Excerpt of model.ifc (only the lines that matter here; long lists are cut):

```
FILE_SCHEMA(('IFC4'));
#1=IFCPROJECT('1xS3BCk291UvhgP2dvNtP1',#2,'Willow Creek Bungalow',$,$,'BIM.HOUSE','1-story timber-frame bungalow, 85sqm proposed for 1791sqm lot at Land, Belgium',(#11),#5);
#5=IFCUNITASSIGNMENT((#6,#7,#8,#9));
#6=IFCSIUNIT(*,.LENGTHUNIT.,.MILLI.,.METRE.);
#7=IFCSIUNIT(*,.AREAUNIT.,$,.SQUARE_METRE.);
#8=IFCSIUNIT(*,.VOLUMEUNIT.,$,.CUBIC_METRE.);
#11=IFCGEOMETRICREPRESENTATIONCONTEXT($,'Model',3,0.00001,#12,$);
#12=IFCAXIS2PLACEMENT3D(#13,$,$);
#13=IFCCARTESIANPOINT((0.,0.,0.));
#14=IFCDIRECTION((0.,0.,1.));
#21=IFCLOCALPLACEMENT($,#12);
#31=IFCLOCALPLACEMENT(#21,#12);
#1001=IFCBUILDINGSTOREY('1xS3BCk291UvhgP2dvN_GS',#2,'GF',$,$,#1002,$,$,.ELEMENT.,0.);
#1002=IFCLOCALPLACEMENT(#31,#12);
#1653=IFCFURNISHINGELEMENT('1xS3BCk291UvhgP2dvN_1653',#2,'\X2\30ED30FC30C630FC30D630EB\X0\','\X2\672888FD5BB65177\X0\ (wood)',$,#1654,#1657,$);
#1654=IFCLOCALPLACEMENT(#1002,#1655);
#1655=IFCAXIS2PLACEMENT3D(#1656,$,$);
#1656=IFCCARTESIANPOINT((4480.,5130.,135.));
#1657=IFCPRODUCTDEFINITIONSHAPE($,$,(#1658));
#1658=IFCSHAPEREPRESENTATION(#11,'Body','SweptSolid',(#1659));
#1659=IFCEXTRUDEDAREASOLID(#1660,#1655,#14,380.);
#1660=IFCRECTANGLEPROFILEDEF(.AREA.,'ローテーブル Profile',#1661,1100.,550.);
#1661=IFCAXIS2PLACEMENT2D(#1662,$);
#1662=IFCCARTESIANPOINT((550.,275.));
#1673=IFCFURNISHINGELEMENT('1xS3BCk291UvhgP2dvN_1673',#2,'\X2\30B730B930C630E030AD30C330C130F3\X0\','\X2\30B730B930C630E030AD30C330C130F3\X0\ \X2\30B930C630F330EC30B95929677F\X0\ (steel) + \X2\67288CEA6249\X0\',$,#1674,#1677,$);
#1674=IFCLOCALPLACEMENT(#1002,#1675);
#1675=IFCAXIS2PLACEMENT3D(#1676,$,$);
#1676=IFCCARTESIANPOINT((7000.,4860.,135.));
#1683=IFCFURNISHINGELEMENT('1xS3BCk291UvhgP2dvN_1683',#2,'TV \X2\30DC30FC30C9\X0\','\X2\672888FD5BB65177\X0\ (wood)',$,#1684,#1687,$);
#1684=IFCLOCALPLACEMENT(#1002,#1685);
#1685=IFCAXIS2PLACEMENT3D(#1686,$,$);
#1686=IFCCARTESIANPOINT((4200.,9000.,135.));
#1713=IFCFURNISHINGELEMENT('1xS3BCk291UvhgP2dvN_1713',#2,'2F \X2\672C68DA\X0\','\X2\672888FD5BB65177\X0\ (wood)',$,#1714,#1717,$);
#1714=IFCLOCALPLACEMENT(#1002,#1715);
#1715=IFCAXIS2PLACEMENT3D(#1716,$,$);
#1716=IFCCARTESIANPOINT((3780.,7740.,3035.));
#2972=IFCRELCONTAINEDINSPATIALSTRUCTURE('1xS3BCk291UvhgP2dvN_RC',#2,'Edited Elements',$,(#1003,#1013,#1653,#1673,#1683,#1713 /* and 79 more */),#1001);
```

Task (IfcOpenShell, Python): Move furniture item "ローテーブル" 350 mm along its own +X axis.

```python
import ifcopenshell
import ifcopenshell.api.geometry
import ifcopenshell.util.placement
import ifcopenshell.util.unit

model = ifcopenshell.open("model.ifc")
unit_scale = ifcopenshell.util.unit.calculate_unit_scale(model)

item = model.by_guid("1xS3BCk291UvhgP2dvN_1653")
matrix = ifcopenshell.util.placement.get_local_placement(item.ObjectPlacement)
matrix[:3, 3] += matrix[:3, 0] * 0.35 / unit_scale
ifcopenshell.api.geometry.edit_object_placement(model, product=item, matrix=matrix, is_si=False)

print(ifcopenshell.util.placement.get_local_placement(item.ObjectPlacement).round(3) + 0.0)

model.write("model_edited.ifc")
```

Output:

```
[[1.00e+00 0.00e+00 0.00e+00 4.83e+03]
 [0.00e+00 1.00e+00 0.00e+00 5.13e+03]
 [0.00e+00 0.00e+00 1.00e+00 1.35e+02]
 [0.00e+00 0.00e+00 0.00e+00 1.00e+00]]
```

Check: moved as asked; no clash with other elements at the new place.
